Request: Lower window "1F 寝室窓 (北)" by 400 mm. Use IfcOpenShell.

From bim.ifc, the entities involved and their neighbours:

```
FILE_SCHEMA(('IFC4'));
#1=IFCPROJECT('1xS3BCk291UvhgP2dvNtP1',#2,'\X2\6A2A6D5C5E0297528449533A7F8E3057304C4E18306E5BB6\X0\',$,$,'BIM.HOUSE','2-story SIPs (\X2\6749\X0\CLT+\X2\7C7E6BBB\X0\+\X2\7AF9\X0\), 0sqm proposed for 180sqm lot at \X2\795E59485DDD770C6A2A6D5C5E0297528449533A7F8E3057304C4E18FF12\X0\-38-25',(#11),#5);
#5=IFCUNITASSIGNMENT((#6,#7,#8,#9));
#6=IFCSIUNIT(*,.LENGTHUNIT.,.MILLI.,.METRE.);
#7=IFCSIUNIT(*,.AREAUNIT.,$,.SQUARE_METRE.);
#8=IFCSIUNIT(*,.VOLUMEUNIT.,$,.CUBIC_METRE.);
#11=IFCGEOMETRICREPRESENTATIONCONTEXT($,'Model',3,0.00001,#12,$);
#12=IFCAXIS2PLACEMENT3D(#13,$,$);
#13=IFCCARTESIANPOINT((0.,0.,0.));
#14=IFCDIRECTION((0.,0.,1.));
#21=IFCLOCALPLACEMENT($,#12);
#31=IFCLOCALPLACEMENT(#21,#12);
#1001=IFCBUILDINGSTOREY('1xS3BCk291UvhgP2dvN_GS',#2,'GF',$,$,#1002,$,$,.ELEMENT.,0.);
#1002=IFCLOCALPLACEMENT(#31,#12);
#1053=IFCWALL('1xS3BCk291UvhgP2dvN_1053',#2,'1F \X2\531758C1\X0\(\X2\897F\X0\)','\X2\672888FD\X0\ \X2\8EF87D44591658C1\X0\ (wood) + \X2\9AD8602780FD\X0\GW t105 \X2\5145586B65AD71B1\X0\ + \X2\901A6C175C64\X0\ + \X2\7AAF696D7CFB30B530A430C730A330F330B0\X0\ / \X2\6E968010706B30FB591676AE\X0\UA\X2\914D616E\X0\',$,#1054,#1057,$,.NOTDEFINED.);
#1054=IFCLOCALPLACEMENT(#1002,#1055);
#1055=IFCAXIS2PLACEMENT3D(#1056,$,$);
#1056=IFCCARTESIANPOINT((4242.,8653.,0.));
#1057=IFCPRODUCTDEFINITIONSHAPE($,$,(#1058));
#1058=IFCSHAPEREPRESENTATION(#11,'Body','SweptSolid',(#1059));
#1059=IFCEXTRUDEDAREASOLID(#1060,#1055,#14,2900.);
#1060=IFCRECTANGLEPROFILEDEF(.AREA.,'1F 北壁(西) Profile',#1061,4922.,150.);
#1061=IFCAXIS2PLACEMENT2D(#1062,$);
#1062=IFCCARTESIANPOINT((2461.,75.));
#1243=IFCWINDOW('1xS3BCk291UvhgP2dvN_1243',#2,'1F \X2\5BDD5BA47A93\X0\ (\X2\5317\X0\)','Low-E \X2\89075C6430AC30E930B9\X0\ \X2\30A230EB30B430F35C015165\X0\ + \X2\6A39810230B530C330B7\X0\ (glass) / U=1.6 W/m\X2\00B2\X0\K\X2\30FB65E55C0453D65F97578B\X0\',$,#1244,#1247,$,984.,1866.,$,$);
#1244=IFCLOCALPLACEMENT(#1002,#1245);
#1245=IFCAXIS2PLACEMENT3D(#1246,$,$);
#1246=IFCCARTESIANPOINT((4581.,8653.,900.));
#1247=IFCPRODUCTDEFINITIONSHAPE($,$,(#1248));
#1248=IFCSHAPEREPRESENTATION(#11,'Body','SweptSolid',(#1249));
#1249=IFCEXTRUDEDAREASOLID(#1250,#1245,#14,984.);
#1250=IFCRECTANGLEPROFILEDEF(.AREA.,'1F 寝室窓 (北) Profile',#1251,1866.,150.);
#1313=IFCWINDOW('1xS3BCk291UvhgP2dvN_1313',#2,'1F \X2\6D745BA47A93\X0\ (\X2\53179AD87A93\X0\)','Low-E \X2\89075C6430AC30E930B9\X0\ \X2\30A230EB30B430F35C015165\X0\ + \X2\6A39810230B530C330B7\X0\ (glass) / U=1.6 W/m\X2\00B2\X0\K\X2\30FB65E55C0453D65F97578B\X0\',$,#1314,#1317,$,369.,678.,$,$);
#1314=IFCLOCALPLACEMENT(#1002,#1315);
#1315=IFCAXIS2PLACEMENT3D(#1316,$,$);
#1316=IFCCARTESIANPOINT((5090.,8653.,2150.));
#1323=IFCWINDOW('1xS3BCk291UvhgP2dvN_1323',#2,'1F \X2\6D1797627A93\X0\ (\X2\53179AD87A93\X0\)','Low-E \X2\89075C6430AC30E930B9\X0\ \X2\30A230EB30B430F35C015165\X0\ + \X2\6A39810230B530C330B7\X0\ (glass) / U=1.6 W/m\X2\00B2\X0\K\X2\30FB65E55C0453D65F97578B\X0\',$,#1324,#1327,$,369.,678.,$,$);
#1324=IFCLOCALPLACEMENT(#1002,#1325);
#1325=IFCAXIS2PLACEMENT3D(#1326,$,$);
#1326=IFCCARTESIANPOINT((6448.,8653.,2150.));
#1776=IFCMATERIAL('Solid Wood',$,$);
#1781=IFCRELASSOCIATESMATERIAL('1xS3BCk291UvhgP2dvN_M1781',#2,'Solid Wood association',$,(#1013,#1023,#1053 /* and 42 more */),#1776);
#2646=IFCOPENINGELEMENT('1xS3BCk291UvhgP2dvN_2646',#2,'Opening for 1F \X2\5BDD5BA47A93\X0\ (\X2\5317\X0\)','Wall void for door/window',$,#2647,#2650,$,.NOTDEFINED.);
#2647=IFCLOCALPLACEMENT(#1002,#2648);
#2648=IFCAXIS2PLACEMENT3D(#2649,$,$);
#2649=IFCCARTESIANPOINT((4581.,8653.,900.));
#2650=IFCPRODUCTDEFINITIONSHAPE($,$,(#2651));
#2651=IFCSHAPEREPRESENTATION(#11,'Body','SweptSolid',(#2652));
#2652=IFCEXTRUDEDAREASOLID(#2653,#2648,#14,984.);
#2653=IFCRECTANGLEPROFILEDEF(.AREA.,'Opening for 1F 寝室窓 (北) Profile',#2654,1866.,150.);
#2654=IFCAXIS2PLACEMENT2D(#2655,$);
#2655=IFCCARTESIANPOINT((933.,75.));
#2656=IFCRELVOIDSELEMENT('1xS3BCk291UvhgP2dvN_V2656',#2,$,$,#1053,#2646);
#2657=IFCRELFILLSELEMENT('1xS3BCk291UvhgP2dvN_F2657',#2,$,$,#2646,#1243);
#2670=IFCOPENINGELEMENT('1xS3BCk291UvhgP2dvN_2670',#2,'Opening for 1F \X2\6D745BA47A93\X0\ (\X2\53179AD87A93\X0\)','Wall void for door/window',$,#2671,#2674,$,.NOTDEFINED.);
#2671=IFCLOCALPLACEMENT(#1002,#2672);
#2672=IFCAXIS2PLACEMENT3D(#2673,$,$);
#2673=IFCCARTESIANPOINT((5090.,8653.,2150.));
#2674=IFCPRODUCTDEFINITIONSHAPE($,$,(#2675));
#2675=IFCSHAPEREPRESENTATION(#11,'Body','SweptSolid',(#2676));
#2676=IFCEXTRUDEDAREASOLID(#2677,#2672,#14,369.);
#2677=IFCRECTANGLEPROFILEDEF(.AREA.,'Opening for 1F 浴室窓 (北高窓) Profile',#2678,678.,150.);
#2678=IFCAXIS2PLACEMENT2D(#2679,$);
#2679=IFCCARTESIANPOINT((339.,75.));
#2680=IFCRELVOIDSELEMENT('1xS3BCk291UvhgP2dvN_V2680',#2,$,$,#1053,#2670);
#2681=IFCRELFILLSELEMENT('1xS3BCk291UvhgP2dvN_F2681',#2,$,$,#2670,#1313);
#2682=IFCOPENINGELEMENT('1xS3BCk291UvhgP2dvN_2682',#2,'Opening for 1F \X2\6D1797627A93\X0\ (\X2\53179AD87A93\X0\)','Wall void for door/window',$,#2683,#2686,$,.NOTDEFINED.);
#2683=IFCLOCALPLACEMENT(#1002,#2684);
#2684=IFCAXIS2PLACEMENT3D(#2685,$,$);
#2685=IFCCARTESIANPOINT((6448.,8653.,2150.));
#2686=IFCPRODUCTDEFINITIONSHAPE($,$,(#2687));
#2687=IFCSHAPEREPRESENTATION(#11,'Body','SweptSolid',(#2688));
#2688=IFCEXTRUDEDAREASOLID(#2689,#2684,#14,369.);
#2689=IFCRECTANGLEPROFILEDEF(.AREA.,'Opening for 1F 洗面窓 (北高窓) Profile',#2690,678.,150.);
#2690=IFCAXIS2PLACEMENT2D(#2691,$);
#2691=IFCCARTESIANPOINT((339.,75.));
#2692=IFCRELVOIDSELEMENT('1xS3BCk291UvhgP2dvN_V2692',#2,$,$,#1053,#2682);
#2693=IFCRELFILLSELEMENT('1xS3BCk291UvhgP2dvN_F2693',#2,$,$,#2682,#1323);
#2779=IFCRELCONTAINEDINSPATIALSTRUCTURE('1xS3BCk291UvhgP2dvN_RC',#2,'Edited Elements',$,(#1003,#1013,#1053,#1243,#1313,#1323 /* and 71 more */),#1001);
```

```python
import numpy as np
import ifcopenshell
import ifcopenshell.api.geometry
import ifcopenshell.util.placement
import ifcopenshell.util.unit

model = ifcopenshell.open("bim.ifc")
unit_scale = ifcopenshell.util.unit.calculate_unit_scale(model)

window = model.by_guid("1xS3BCk291UvhgP2dvN_1243")
opening = window.FillsVoids[0].RelatingOpeningElement
dz = -0.4 / unit_scale

shift = np.array([0.0, 0.0, dz])
# The window is not placed relative to its opening, so move both.
for product in (opening, window):
    matrix = ifcopenshell.util.placement.get_local_placement(product.ObjectPlacement)
    matrix[:3, 3] += shift
    ifcopenshell.api.geometry.edit_object_placement(model, product=product, matrix=matrix, is_si=False)

print(f"moved by {dz * unit_scale:+.3f} m")

model.write("bim-out.ifc")
```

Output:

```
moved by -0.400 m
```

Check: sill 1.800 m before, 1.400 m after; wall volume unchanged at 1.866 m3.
